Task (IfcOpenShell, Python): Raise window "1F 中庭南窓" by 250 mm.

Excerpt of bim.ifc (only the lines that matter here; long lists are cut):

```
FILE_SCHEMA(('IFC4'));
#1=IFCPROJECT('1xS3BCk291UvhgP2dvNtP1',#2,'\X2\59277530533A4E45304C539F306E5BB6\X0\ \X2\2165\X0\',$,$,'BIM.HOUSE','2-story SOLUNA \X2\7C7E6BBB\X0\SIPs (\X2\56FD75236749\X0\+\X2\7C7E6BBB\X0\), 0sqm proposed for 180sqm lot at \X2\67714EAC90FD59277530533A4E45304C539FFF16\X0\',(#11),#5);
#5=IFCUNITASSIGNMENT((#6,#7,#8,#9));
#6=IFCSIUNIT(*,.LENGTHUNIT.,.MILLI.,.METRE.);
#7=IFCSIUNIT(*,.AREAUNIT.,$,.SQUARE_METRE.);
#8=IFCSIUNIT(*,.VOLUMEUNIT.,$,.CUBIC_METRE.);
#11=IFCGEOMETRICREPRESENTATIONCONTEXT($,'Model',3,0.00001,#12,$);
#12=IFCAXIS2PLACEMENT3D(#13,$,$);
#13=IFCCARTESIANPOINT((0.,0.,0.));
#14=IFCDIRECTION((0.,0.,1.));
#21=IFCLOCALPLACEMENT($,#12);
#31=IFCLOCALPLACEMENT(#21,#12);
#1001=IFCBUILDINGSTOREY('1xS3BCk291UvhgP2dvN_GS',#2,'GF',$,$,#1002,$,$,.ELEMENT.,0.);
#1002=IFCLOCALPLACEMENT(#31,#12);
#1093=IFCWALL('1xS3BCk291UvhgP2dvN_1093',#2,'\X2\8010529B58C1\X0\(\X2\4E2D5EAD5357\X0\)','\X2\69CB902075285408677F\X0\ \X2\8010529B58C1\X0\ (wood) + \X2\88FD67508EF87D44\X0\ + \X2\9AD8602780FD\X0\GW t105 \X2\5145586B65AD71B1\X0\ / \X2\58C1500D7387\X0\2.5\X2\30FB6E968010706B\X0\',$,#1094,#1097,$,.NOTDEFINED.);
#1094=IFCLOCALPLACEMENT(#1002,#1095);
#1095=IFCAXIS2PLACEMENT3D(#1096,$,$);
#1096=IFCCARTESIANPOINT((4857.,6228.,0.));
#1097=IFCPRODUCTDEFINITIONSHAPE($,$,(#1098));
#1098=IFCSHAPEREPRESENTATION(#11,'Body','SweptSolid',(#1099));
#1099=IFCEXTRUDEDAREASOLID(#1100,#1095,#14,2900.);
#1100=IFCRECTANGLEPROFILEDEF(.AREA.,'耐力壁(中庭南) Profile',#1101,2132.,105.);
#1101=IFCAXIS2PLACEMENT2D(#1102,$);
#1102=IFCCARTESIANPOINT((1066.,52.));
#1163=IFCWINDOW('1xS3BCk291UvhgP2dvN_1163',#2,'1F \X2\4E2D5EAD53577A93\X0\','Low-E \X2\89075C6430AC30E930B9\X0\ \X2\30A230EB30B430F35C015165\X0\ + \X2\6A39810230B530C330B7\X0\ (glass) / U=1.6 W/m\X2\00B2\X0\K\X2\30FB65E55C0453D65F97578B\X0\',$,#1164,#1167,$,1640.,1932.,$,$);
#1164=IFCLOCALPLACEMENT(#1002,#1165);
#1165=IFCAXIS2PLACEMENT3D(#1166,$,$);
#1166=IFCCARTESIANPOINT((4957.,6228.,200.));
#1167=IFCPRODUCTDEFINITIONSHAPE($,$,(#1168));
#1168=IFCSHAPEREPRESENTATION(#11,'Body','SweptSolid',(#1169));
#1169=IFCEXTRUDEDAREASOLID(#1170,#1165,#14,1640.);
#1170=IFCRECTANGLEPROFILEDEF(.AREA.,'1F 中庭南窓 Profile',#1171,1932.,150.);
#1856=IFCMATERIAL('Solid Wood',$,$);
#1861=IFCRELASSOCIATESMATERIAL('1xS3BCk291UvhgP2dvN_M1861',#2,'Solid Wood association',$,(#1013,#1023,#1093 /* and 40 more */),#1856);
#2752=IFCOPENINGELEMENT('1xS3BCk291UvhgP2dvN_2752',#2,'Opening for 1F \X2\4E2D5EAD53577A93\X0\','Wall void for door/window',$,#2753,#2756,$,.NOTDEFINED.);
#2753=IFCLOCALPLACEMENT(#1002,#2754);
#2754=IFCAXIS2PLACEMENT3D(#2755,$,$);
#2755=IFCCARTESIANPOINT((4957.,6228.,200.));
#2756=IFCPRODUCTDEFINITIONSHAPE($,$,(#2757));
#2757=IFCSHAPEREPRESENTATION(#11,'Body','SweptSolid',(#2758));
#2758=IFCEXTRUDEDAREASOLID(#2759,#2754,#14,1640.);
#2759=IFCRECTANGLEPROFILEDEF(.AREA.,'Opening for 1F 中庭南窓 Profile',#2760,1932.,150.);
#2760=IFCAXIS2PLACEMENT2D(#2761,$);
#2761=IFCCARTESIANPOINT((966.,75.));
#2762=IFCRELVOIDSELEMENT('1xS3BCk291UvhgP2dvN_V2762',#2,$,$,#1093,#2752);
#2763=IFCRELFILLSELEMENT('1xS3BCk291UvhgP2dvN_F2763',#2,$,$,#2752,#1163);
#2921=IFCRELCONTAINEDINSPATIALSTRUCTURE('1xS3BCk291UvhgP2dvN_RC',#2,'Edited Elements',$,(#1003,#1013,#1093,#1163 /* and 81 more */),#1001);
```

```python
import numpy as np
import ifcopenshell
import ifcopenshell.api.geometry
import ifcopenshell.util.placement
import ifcopenshell.util.unit

model = ifcopenshell.open("bim.ifc")
unit_scale = ifcopenshell.util.unit.calculate_unit_scale(model)

window = model.by_guid("1xS3BCk291UvhgP2dvN_1163")
opening = window.FillsVoids[0].RelatingOpeningElement
dz = 0.25 / unit_scale

shift = np.array([0.0, 0.0, dz])
# The window is not placed relative to its opening, so move both.
for product in (opening, window):
    matrix = ifcopenshell.util.placement.get_local_placement(product.ObjectPlacement)
    matrix[:3, 3] += shift
    ifcopenshell.api.geometry.edit_object_placement(model, product=product, matrix=matrix, is_si=False)

print(f"moved by {dz * unit_scale:+.3f} m")

model.write("bim_v2.ifc")
```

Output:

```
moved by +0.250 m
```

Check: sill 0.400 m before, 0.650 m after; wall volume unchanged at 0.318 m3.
